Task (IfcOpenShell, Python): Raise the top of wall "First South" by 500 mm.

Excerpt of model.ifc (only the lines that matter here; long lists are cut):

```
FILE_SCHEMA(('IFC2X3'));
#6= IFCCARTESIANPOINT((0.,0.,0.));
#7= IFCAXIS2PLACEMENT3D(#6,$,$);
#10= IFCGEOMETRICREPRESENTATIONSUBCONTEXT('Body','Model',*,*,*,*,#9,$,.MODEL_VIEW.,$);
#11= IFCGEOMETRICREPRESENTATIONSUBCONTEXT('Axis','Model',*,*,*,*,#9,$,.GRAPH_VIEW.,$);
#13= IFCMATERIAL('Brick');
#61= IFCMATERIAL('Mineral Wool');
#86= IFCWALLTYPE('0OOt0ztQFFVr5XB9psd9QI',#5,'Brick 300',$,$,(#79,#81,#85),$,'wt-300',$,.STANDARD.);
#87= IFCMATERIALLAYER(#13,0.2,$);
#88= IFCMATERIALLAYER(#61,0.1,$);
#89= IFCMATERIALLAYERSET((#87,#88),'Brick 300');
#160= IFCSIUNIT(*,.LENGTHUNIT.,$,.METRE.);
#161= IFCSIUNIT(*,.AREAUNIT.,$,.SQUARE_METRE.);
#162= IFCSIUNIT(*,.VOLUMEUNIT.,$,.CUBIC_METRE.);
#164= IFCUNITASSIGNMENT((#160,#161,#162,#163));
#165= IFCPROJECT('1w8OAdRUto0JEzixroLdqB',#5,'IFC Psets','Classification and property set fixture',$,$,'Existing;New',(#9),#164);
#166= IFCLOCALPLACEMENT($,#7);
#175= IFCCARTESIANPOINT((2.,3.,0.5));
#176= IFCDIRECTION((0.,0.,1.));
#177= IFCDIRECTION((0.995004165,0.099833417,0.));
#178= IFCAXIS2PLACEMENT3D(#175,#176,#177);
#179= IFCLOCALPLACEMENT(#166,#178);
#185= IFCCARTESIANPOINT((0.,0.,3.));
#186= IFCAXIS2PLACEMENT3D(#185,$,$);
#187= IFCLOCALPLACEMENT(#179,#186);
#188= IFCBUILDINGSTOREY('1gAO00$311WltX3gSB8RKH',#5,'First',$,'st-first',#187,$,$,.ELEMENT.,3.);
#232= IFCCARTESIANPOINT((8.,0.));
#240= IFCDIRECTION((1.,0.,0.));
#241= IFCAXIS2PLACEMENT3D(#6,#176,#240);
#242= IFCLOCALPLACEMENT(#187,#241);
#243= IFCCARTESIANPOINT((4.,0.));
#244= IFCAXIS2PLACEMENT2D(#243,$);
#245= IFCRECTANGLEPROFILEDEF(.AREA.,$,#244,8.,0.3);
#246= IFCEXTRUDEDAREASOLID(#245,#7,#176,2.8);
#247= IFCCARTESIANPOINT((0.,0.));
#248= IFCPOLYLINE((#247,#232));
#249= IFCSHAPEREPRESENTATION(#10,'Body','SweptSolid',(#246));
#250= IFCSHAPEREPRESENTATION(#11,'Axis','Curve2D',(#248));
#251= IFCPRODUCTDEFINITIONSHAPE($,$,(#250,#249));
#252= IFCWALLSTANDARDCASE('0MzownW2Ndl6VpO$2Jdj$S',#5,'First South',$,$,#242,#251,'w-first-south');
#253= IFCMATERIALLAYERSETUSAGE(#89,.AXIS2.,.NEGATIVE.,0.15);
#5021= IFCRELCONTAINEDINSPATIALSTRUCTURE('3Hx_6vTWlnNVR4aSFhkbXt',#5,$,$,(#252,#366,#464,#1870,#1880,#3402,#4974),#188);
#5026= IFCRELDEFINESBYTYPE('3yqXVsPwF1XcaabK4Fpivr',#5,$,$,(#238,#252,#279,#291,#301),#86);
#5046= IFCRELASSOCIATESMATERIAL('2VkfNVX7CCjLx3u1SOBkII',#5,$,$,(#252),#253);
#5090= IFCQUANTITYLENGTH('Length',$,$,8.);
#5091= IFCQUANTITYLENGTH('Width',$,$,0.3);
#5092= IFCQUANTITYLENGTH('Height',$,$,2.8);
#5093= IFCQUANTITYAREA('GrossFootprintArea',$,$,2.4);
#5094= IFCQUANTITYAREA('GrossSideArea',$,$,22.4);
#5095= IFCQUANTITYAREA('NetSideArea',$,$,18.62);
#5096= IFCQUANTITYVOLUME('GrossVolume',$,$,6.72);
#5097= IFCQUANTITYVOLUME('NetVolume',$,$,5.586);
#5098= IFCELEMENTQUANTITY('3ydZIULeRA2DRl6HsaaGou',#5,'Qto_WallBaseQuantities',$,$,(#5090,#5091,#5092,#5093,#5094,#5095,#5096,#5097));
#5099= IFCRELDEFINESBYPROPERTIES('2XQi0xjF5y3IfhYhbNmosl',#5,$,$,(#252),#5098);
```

```python
import ifcopenshell
import ifcopenshell.api.pset
import ifcopenshell.geom
import ifcopenshell.util.element
import ifcopenshell.util.representation
import ifcopenshell.util.shape
import ifcopenshell.util.unit

model = ifcopenshell.open("model.ifc")
unit_scale = ifcopenshell.util.unit.calculate_unit_scale(model)
area_scale = ifcopenshell.util.unit.calculate_unit_scale(model, "AREAUNIT")
volume_scale = ifcopenshell.util.unit.calculate_unit_scale(model, "VOLUMEUNIT")
settings = ifcopenshell.geom.settings()


def volume(element):
    """Net volume in cubic metres, openings subtracted."""
    shape = ifcopenshell.geom.create_shape(settings, element)
    return ifcopenshell.util.shape.get_volume(shape.geometry)


wall = model.by_guid("0MzownW2Ndl6VpO$2Jdj$S")
before = volume(wall)

body = ifcopenshell.util.representation.get_representation(wall, "Model", "Body")
solid = body.Items[0]
old_height = solid.Depth
solid.Depth += 0.5
after = volume(wall)
thickness = 0.3  # wall thickness in metres

# Update the stored height, areas and volumes.
qto = model.by_id(ifcopenshell.util.element.get_pset(wall, "Qto_WallBaseQuantities", should_inherit=False)["id"])
ifcopenshell.api.pset.edit_qto(model, qto=qto, properties={
    "Height": solid.Depth,
    "GrossSideArea": ifcopenshell.util.element.get_pset(wall, "Qto_WallBaseQuantities", "GrossSideArea") * solid.Depth / old_height,
    "NetSideArea": after / thickness / area_scale,
    "GrossVolume": ifcopenshell.util.element.get_pset(wall, "Qto_WallBaseQuantities", "GrossVolume") * solid.Depth / old_height,
    "NetVolume": after / volume_scale,
})

print(f"height {old_height:g} -> {solid.Depth:g}, volume {before:.3f} -> {after:.3f} m3")

model.write("model_v2.ifc")
```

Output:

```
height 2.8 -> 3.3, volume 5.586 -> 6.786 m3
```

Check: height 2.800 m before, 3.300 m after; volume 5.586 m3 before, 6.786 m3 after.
